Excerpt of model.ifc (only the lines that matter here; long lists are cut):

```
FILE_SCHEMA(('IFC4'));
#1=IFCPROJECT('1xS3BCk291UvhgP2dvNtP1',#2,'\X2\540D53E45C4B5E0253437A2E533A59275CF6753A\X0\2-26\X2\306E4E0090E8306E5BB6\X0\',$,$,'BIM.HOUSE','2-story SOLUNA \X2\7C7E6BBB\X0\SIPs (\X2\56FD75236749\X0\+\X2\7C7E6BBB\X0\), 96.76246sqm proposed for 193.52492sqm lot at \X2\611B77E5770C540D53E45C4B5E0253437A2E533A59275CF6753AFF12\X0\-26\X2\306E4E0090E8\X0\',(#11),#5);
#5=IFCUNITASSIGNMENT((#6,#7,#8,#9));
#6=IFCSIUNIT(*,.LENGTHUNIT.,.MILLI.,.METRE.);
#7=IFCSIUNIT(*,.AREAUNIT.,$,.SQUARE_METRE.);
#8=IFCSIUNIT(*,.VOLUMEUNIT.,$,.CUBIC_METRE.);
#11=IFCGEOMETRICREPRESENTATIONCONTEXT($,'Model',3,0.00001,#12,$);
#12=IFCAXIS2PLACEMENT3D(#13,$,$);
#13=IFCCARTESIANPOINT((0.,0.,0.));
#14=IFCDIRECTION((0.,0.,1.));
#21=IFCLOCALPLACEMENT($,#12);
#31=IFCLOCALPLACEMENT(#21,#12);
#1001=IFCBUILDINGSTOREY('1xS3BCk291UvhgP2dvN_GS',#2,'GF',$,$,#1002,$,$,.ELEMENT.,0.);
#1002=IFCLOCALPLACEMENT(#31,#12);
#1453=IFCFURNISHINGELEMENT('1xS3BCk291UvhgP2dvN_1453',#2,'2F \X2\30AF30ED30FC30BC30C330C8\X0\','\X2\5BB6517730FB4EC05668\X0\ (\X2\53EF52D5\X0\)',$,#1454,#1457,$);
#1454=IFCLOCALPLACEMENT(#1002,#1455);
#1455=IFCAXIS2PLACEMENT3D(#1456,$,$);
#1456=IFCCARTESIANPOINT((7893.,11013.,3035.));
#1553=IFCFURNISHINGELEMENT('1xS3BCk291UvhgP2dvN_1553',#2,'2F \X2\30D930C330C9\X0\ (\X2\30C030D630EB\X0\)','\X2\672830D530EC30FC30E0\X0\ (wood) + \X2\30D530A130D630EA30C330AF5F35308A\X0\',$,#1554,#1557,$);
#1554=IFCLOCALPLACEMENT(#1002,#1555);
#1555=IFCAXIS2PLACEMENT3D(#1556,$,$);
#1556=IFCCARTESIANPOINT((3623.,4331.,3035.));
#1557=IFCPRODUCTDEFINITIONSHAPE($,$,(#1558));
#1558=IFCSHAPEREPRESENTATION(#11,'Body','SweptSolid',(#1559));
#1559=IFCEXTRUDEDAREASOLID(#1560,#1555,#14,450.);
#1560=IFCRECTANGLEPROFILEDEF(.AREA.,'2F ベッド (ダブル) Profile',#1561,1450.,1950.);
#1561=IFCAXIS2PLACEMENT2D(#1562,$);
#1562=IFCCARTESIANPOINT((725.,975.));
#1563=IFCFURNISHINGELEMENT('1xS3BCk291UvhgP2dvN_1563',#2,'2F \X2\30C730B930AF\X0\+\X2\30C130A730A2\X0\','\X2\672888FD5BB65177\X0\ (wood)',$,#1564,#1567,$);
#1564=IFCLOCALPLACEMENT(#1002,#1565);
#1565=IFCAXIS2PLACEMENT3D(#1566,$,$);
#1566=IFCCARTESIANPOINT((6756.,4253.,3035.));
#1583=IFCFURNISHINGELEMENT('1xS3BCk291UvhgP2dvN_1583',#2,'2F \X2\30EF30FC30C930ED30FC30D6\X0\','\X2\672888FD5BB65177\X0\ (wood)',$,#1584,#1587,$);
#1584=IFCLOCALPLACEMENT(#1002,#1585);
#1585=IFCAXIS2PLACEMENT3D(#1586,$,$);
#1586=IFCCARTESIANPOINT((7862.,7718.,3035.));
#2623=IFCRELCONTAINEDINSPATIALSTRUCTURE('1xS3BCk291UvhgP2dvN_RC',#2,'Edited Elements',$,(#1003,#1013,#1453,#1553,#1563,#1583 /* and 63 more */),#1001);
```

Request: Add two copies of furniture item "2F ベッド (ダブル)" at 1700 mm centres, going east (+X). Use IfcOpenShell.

```python
import numpy as np
import ifcopenshell
import ifcopenshell.api.geometry
import ifcopenshell.api.root
import ifcopenshell.util.element
import ifcopenshell.util.placement

model = ifcopenshell.open("model.ifc")


def reuse_history(source, copy):
    """copy_class also copies each property set's owner history, people and application; keep the originals."""
    for rel in copy.IsDefinedBy:
        if rel.is_a("IfcRelDefinesByProperties") and (history := rel.RelatingPropertyDefinition.OwnerHistory):
            rel.RelatingPropertyDefinition.OwnerHistory = source.OwnerHistory
            ifcopenshell.util.element.remove_deep2(model, history)


source = model.by_guid("1xS3BCk291UvhgP2dvN_1553")
base = ifcopenshell.util.placement.get_local_placement(source.ObjectPlacement)
step = np.array([1.0, 0.0, 0.0]) * 1700.0

for i in range(1, 3):
    copy = ifcopenshell.api.root.copy_class(model, product=source)
    copy.Representation = ifcopenshell.util.element.copy_deep(
        model, source.Representation, exclude=["IfcGeometricRepresentationContext", "IfcRepresentationMap"]
    )
    reuse_history(source, copy)
    matrix = base.copy()
    matrix[:3, 3] += i * step
    print("added at", matrix[:3, 3].round(3) + 0.0)
    ifcopenshell.api.geometry.edit_object_placement(model, product=copy, matrix=matrix, is_si=False)

model.write("model_edited.ifc")
```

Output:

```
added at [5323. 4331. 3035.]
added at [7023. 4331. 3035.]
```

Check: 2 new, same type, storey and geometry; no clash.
